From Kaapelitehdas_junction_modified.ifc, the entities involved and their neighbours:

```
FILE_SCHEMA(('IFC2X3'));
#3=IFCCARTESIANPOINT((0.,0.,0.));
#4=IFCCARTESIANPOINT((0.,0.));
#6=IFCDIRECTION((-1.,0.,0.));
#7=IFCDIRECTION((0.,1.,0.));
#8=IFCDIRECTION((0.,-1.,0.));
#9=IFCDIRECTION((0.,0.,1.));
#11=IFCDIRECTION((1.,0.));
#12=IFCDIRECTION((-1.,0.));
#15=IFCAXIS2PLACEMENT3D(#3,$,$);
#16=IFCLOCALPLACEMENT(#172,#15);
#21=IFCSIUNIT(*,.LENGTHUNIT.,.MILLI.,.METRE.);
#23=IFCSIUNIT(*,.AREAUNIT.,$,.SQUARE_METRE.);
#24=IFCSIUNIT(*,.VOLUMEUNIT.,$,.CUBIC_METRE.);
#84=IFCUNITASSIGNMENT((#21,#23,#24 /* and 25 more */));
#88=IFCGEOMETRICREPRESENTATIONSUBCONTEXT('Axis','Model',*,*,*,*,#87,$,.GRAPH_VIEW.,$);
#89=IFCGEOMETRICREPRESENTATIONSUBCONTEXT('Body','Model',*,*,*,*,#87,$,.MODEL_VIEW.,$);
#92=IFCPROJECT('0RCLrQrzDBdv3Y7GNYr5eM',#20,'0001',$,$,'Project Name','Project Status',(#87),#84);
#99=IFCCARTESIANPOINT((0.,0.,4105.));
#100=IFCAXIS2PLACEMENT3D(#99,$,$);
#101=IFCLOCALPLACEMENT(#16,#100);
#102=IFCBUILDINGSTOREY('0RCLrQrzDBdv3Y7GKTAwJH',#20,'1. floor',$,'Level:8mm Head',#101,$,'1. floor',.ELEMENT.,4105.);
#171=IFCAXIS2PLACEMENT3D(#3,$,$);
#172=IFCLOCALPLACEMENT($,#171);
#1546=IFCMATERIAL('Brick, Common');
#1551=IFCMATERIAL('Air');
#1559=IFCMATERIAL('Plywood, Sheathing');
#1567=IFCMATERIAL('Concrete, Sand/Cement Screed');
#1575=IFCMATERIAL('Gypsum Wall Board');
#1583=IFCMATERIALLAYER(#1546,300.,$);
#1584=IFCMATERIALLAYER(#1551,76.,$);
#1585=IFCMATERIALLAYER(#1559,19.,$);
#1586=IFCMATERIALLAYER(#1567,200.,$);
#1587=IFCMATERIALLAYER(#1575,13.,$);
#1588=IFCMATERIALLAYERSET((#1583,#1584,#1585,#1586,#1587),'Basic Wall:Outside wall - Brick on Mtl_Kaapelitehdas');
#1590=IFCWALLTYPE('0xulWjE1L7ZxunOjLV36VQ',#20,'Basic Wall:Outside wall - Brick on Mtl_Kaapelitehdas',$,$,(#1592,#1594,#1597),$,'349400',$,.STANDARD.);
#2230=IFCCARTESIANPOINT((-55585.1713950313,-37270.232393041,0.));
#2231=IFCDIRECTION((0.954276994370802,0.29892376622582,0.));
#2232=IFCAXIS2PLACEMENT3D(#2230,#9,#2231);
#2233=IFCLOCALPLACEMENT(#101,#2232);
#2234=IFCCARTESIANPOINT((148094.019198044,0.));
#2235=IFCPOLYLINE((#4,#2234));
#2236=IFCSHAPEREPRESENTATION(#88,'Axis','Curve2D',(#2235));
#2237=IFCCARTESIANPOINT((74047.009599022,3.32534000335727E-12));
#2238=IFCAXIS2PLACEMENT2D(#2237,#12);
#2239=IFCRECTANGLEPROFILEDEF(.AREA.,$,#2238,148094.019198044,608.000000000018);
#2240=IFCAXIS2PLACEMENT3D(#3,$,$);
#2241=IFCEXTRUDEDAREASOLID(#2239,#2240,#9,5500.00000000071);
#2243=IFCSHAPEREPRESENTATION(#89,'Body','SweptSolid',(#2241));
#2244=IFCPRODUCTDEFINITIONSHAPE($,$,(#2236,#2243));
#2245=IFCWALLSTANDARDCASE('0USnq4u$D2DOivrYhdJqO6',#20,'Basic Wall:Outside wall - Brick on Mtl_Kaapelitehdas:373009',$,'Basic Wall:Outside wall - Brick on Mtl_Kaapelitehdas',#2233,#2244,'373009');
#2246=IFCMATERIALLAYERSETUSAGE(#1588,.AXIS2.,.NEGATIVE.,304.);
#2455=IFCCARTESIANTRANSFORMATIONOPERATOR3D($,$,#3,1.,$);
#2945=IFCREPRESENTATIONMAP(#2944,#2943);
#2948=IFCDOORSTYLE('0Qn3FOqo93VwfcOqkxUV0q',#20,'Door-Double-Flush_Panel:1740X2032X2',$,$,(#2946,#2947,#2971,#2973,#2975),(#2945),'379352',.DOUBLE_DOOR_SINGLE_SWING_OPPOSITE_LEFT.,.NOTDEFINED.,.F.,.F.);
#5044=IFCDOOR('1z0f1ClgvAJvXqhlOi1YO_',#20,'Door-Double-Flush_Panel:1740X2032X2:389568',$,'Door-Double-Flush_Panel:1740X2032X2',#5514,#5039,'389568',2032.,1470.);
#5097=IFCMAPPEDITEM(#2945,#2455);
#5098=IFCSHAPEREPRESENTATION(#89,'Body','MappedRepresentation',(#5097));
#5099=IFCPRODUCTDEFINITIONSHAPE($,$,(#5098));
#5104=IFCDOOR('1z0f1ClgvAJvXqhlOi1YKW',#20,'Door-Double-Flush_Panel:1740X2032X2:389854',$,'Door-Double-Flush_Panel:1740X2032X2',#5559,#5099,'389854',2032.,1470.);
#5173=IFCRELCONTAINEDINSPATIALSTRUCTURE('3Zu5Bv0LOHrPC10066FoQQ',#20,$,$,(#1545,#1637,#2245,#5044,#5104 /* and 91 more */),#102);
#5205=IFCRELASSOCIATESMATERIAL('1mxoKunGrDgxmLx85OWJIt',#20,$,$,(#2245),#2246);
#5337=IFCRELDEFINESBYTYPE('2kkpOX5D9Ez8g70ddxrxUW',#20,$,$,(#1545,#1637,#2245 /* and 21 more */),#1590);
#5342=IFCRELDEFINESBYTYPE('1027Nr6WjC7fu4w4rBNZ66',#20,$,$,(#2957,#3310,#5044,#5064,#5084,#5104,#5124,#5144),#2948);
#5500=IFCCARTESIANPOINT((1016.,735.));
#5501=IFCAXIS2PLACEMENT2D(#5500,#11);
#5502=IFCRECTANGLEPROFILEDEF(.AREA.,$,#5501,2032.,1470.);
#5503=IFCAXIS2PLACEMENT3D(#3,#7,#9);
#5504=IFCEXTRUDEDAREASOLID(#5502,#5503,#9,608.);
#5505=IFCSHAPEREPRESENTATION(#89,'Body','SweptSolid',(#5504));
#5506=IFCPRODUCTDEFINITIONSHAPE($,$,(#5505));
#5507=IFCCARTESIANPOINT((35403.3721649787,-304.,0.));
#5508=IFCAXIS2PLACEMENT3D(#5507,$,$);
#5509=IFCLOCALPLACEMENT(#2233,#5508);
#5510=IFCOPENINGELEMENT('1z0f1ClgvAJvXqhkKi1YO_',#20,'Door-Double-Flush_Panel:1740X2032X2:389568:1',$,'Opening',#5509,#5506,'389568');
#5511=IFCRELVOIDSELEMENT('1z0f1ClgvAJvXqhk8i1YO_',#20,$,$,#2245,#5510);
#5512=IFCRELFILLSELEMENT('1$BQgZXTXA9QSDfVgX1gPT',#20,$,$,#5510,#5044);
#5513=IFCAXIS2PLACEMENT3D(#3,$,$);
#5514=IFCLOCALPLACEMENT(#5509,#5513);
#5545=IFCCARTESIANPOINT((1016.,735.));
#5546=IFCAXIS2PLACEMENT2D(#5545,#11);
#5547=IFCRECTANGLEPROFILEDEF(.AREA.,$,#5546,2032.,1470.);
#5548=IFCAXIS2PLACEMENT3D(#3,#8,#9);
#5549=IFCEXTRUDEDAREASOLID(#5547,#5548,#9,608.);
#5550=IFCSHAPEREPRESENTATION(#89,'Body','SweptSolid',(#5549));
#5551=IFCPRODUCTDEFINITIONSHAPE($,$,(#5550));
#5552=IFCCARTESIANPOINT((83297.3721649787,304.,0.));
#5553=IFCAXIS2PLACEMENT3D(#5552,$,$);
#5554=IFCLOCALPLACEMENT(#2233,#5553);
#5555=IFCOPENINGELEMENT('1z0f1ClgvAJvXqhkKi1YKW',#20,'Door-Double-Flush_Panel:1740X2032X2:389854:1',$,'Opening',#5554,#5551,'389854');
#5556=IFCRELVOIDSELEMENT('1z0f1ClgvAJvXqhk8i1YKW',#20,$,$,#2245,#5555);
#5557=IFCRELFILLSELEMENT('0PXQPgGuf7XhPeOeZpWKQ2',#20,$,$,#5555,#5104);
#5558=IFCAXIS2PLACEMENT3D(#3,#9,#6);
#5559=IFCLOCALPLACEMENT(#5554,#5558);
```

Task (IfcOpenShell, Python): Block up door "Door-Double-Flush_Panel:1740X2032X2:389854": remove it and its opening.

```python
import ifcopenshell
import ifcopenshell.api.feature
import ifcopenshell.api.root
import ifcopenshell.geom
import ifcopenshell.util.shape

model = ifcopenshell.open("Kaapelitehdas_junction_modified.ifc")
settings = ifcopenshell.geom.settings()


def volume(element):
    """Net volume in cubic metres, openings subtracted."""
    shape = ifcopenshell.geom.create_shape(settings, element)
    return ifcopenshell.util.shape.get_volume(shape.geometry)


door = model.by_guid("1z0f1ClgvAJvXqhlOi1YKW")
opening = door.FillsVoids[0].RelatingOpeningElement
wall = opening.VoidsElements[0].RelatingBuildingElement
before = volume(wall)

ifcopenshell.api.root.remove_product(model, product=door)
ifcopenshell.api.feature.remove_feature(model, feature=opening)

after = volume(wall)

print(f"wall volume {before:.3f} -> {after:.3f} m3")

model.write("Kaapelitehdas_junction_modified_updated.ifc")
```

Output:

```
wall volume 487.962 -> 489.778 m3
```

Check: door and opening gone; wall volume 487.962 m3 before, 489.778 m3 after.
